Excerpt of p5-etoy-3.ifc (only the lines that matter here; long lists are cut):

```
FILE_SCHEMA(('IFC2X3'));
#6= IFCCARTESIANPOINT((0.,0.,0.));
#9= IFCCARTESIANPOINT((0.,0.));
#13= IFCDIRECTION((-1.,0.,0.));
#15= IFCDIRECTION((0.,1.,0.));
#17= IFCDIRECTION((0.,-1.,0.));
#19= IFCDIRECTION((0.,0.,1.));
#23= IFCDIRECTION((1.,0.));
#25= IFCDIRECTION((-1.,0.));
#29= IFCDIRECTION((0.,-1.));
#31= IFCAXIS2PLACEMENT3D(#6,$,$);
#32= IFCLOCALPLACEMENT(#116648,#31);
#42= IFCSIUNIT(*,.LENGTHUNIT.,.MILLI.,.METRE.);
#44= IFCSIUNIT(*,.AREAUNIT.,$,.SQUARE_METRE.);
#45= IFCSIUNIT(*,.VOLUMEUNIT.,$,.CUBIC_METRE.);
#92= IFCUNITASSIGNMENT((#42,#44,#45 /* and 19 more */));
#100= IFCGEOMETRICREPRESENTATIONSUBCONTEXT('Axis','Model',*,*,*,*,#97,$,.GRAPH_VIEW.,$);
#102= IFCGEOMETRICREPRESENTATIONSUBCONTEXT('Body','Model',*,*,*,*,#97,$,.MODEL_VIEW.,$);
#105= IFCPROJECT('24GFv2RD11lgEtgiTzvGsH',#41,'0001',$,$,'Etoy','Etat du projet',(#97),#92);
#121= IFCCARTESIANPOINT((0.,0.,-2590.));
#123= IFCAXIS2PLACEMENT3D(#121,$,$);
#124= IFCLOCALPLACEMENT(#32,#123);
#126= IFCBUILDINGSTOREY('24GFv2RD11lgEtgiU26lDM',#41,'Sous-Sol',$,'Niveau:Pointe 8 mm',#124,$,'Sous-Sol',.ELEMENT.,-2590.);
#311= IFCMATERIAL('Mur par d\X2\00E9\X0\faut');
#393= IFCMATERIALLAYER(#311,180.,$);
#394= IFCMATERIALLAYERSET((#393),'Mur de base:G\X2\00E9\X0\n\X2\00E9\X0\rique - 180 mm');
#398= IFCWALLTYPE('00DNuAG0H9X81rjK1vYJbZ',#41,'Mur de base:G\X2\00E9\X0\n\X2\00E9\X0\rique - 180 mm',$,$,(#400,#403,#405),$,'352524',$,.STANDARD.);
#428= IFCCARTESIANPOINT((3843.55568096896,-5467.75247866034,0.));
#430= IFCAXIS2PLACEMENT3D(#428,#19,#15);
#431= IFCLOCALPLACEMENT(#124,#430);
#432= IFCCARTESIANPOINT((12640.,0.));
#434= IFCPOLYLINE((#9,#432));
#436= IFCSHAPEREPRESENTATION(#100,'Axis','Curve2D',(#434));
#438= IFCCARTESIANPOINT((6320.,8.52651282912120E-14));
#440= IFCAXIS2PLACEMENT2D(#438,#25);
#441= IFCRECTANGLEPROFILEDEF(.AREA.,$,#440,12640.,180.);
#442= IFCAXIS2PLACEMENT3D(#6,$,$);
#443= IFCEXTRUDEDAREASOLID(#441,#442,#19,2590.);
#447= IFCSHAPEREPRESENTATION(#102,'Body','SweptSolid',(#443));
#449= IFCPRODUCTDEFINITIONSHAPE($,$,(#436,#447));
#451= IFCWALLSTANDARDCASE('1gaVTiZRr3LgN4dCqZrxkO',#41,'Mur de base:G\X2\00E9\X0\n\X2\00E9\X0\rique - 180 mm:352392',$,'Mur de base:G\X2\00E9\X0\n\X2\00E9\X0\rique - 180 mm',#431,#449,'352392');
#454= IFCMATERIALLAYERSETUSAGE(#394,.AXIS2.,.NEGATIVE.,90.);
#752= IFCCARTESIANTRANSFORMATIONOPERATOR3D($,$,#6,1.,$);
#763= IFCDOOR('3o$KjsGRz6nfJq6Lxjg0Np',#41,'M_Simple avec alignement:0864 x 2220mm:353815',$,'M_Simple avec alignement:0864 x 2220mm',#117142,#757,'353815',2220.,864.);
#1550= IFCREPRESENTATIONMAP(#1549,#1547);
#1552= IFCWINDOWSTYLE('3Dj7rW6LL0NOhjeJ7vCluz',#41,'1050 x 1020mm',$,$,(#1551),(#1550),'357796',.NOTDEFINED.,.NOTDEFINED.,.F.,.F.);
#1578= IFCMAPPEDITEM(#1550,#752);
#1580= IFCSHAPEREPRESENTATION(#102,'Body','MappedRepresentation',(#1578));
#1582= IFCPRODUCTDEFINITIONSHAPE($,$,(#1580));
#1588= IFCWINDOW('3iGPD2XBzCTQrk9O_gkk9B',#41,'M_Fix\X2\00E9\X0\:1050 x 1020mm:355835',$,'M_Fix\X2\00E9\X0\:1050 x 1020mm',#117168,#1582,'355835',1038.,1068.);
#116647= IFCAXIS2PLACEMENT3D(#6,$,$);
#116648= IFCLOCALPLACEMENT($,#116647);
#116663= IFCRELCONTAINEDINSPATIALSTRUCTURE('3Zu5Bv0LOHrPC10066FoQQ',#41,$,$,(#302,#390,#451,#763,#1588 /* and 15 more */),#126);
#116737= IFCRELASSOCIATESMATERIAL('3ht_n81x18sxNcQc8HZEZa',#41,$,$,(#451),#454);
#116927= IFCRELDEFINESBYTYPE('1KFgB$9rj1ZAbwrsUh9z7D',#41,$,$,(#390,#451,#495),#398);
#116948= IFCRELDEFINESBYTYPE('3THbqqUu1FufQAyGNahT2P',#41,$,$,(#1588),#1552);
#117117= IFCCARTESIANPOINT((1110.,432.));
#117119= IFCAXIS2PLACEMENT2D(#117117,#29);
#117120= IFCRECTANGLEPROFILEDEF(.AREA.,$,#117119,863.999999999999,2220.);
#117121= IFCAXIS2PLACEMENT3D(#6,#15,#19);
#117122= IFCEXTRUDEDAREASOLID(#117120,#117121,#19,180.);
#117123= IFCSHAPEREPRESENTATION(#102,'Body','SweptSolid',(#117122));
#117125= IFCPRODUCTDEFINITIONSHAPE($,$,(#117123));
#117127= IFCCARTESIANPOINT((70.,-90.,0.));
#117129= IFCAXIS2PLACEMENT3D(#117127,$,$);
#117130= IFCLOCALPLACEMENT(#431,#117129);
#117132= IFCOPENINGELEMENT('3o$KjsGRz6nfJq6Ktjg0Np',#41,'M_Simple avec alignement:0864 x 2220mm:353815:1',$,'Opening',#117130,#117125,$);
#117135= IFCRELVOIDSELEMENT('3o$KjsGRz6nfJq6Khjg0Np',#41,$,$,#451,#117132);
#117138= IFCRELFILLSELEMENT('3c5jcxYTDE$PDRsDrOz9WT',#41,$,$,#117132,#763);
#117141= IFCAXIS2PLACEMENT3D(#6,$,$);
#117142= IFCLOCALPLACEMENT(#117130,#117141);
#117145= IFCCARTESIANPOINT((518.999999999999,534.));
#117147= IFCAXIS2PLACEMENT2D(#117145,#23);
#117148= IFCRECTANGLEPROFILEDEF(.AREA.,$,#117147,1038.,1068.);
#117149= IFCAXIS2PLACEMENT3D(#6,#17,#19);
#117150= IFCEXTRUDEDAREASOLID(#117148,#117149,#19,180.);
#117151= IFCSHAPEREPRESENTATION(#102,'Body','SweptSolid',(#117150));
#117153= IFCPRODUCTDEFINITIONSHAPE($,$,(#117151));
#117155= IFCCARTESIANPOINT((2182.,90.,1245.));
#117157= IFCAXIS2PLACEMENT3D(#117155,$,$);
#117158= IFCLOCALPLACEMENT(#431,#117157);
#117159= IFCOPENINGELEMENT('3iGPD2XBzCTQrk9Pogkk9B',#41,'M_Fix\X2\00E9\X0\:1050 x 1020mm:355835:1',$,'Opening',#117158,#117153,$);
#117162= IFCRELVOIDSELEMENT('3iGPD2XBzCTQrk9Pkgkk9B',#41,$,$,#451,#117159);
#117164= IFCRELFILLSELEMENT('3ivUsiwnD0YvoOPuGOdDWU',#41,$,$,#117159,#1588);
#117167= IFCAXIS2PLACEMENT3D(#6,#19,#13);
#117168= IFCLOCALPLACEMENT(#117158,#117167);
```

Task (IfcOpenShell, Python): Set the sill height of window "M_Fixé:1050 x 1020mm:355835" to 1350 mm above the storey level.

```python
import numpy as np
import ifcopenshell
import ifcopenshell.api.geometry
import ifcopenshell.geom
import ifcopenshell.util.element
import ifcopenshell.util.placement
import ifcopenshell.util.shape
import ifcopenshell.util.unit

model = ifcopenshell.open("p5-etoy-3.ifc")
unit_scale = ifcopenshell.util.unit.calculate_unit_scale(model)

window = model.by_id(1588)
opening = window.FillsVoids[0].RelatingOpeningElement
storey = ifcopenshell.util.element.get_container(window, ifc_class="IfcBuildingStorey")
level = ifcopenshell.util.placement.get_local_placement(storey.ObjectPlacement)[2, 3]

# The opening's origin need not be at the sill, so measure its lowest point.
shape = ifcopenshell.geom.create_shape(ifcopenshell.geom.settings(), opening)
bottom = ifcopenshell.util.shape.get_shape_bottom_elevation(shape, shape.geometry) / unit_scale
dz = level + 1350.0 - bottom

shift = np.array([0.0, 0.0, dz])
# The window is placed relative to its opening, so it follows when the opening moves.
matrix = ifcopenshell.util.placement.get_local_placement(opening.ObjectPlacement)
matrix[:3, 3] += shift
ifcopenshell.api.geometry.edit_object_placement(
    model, product=opening, matrix=matrix, is_si=False, should_transform_children=True
)

print(f"moved by {dz * unit_scale:+.3f} m")

model.write("p5-etoy-3_rev.ifc")
```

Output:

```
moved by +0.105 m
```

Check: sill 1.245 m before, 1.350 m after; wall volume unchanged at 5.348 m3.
